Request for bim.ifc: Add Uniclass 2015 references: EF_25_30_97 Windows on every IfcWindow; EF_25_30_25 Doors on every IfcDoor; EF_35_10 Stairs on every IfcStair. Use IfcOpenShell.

First a look at what the model holds.

```python
import ifcopenshell

model = ifcopenshell.open("bim.ifc")
print(model.schema)
print("classifications:", [c.Name for c in model.by_type("IfcClassification")])
for ifc_class in ("IfcDoor", "IfcRoof", "IfcStair", "IfcWall", "IfcWindow"):
    print(ifc_class, len(model.by_type(ifc_class)))
```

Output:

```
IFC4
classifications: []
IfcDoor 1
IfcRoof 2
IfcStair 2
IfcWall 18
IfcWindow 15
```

```python
import ifcopenshell
import ifcopenshell.api.classification

model = ifcopenshell.open("bim.ifc")

system = ifcopenshell.api.classification.add_classification(model, classification="Uniclass 2015")

codes = {
    "IfcWindow": ("EF_25_30_97", "Windows"),
    "IfcDoor": ("EF_25_30_25", "Doors"),
    "IfcStair": ("EF_35_10", "Stairs"),
}
for ifc_class, (code, name) in codes.items():
    products = model.by_type(ifc_class)
    ifcopenshell.api.classification.add_reference(
        model, products=products, classification=system, identification=code, name=name
    )
    print(code, len(products))

model.write("bim-out.ifc")
```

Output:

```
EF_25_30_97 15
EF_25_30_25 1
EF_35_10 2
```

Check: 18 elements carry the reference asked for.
